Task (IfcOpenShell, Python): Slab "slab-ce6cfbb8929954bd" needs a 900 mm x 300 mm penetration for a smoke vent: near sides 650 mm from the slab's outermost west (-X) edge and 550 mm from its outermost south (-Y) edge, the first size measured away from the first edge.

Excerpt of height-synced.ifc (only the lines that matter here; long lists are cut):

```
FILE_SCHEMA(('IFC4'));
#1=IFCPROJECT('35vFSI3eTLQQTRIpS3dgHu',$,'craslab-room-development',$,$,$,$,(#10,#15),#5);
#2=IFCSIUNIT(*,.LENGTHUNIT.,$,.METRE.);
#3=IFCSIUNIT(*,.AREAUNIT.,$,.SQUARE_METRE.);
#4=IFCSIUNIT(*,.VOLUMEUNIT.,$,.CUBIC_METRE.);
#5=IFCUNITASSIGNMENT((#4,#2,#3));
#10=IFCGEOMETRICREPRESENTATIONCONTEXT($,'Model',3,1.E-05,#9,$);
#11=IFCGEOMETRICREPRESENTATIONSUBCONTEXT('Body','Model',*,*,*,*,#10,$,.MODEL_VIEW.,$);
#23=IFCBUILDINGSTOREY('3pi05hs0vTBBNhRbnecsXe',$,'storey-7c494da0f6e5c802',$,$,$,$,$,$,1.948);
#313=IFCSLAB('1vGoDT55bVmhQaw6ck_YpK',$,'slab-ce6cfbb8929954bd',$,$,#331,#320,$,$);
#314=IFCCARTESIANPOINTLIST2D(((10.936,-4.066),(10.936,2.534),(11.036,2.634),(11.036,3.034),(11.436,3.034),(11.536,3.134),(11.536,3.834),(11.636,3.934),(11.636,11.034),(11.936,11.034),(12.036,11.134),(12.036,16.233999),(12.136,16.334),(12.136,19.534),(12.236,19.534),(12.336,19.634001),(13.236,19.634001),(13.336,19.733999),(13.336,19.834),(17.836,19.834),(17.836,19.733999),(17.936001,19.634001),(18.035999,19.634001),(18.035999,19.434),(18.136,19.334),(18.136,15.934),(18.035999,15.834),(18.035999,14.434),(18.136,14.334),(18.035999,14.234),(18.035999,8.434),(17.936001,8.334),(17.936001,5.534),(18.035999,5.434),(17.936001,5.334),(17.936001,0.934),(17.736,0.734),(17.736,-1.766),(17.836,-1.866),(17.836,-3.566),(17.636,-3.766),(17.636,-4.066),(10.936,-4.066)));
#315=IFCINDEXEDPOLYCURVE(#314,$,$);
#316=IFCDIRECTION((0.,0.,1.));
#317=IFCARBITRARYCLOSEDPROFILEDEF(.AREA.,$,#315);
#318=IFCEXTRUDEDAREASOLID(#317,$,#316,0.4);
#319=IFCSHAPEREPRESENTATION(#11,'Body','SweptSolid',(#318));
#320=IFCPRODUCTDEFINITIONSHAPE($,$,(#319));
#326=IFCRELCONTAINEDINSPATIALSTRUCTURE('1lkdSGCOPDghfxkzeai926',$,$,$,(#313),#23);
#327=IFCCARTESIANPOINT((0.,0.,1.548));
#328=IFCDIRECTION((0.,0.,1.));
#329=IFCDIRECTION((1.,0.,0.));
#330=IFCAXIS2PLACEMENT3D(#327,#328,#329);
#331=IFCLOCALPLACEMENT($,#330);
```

```python
import numpy as np
import ifcopenshell
import ifcopenshell.api.feature
import ifcopenshell.api.geometry
import ifcopenshell.api.root
import ifcopenshell.geom
import ifcopenshell.util.placement
import ifcopenshell.util.representation
import ifcopenshell.util.shape
import ifcopenshell.util.unit

model = ifcopenshell.open("height-synced.ifc")
unit_scale = ifcopenshell.util.unit.calculate_unit_scale(model)
settings = ifcopenshell.geom.settings()


def volume(element):
    """Net volume in cubic metres, openings subtracted."""
    shape = ifcopenshell.geom.create_shape(settings, element)
    return ifcopenshell.util.shape.get_volume(shape.geometry)


slab = model.by_id(313)
before = volume(slab)

# Extent in the slab's own axes, in metres. The edges named are its -X and -Y sides.
slab_shape = ifcopenshell.geom.create_shape(settings, slab)
vertices = ifcopenshell.util.shape.get_vertices(slab_shape.geometry)
x_min, y_min, bottom = vertices.min(axis=0)
top = vertices[:, 2].max()

opening = ifcopenshell.api.root.create_entity(model, ifc_class="IfcOpeningElement", name="Smoke vent opening", predefined_type="OPENING")
context = ifcopenshell.util.representation.get_context(model, "Model", "Body", "MODEL_VIEW")
width, depth = 0.9, 0.3
outline = [(0.0, 0.0), (width, 0.0), (width, depth), (0.0, depth), (0.0, 0.0)]
# Overshoot both faces by 50 mm so the cut is clean.
shape = ifcopenshell.api.geometry.add_slab_representation(
    model, context=context, depth=top - bottom + 0.1, polyline=outline
)
ifcopenshell.api.geometry.assign_representation(model, product=opening, representation=shape)

matrix = ifcopenshell.util.placement.get_local_placement(slab.ObjectPlacement)
matrix[:, 3] = matrix @ np.append(np.array([x_min + 0.65, y_min + 0.55, bottom - 0.05]) / unit_scale, 1.0)
ifcopenshell.api.geometry.edit_object_placement(model, product=opening, matrix=matrix, is_si=False)
ifcopenshell.api.feature.add_feature(model, feature=opening, element=slab)

after = volume(slab)

print(f"slab volume {before:.3f} -> {after:.3f} m3")

model.write("height-synced_updated.ifc")
```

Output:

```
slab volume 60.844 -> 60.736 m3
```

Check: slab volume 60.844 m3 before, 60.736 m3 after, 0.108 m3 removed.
